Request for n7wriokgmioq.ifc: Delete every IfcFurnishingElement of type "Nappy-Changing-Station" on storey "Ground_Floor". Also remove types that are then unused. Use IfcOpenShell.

First a look at what the model holds.

```python
import ifcopenshell
import ifcopenshell.util.element

model = ifcopenshell.open("n7wriokgmioq.ifc")
print(model.schema)
storey = next(s for s in model.by_type("IfcBuildingStorey") if s.Name == "Ground_Floor")
furniture = [e for e in ifcopenshell.util.element.get_decomposition(storey) if e.is_a("IfcFurnishingElement")]
seen = {}
for e in furniture:
    element_type = ifcopenshell.util.element.get_type(e)
    name = element_type.Name if element_type not in (None, e) else None
    seen[name] = seen.get(name, 0) + 1
for name, count in sorted(seen.items(), key=str):
    print(count, "x", name)
```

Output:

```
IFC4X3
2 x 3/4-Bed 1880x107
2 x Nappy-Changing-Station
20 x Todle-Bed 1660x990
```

```python
import ifcopenshell
import ifcopenshell.api.root
import ifcopenshell.util.element

model = ifcopenshell.open("n7wriokgmioq.ifc")

storey = next(s for s in model.by_type("IfcBuildingStorey") if s.Name == "Ground_Floor")
furniture = [e for e in ifcopenshell.util.element.get_decomposition(storey) if e.is_a("IfcFurnishingElement")]
targets = [e for e in furniture if (t := ifcopenshell.util.element.get_type(e)) not in (None, e) and t.Name == "Nappy-Changing-Station"]
types = {ifcopenshell.util.element.get_type(e) for e in targets} - {None, *targets}

for e in targets:
    ifcopenshell.api.root.remove_product(model, product=e)
print(len(targets), "removed")

unused = [t for t in types if not ifcopenshell.util.element.get_types(t)]
for t in unused:
    ifcopenshell.api.root.remove_product(model, product=t)
print(len(unused), "unused types removed")

model.write("n7wriokgmioq_v2.ifc")
```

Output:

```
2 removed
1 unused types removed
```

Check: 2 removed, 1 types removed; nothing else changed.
